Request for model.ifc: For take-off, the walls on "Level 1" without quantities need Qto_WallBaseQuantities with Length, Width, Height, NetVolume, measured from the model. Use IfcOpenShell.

First a look at what the model holds.

```python
import ifcopenshell
import ifcopenshell.util.element
import ifcopenshell.util.unit

model = ifcopenshell.open("model.ifc")
print(model.schema)
for unit_type in ("LENGTHUNIT", "AREAUNIT", "VOLUMEUNIT"):
    print(unit_type, ifcopenshell.util.unit.calculate_unit_scale(model, unit_type))
storey = next(s for s in model.by_type("IfcBuildingStorey") if s.Name == "Level 1")
walls = [e for e in ifcopenshell.util.element.get_decomposition(storey) if e.is_a("IfcWall")]
for e in sorted(walls, key=lambda e: e.id()):
    print(e.id(), e.is_a(), e.Name, list(ifcopenshell.util.element.get_psets(e, qtos_only=True)), sep=" | ")
```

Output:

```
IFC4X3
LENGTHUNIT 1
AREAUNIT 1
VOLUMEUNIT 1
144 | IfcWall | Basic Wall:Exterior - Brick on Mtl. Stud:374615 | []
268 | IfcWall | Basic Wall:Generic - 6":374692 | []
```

```python
import ifcopenshell
import ifcopenshell.api.pset
import ifcopenshell.geom
import ifcopenshell.util.element
import ifcopenshell.util.shape
import ifcopenshell.util.unit

model = ifcopenshell.open("model.ifc")
unit_scale = ifcopenshell.util.unit.calculate_unit_scale(model)
volume_scale = ifcopenshell.util.unit.calculate_unit_scale(model, "VOLUMEUNIT")
settings = ifcopenshell.geom.settings()

storey = next(s for s in model.by_type("IfcBuildingStorey") if s.Name == "Level 1")
walls = [e for e in ifcopenshell.util.element.get_decomposition(storey) if e.is_a("IfcWall")]

for e in sorted(walls, key=lambda e: e.id()):
    if ifcopenshell.util.element.get_psets(e, qtos_only=True, should_inherit=False):
        continue
    # Geometry comes back in metres, in the element's own axes.
    shape = ifcopenshell.geom.create_shape(settings, e)
    values = {
        "Length": ifcopenshell.util.shape.get_x(shape.geometry) / unit_scale,
        "Width": ifcopenshell.util.shape.get_y(shape.geometry) / unit_scale,
        "Height": ifcopenshell.util.shape.get_z(shape.geometry) / unit_scale,
        "NetVolume": ifcopenshell.util.shape.get_volume(shape.geometry) / volume_scale,
    }
    qto = ifcopenshell.api.pset.add_qto(model, product=e, name="Qto_WallBaseQuantities")
    ifcopenshell.api.pset.edit_qto(model, qto=qto, properties=values)
    print(e.id(), {k: round(v, 3) for k, v in values.items()})

model.write("model_updated.ifc")
```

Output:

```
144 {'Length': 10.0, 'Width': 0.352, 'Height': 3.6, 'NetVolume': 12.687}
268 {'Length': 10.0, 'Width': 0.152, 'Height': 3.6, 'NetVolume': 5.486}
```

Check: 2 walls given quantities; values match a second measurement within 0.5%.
